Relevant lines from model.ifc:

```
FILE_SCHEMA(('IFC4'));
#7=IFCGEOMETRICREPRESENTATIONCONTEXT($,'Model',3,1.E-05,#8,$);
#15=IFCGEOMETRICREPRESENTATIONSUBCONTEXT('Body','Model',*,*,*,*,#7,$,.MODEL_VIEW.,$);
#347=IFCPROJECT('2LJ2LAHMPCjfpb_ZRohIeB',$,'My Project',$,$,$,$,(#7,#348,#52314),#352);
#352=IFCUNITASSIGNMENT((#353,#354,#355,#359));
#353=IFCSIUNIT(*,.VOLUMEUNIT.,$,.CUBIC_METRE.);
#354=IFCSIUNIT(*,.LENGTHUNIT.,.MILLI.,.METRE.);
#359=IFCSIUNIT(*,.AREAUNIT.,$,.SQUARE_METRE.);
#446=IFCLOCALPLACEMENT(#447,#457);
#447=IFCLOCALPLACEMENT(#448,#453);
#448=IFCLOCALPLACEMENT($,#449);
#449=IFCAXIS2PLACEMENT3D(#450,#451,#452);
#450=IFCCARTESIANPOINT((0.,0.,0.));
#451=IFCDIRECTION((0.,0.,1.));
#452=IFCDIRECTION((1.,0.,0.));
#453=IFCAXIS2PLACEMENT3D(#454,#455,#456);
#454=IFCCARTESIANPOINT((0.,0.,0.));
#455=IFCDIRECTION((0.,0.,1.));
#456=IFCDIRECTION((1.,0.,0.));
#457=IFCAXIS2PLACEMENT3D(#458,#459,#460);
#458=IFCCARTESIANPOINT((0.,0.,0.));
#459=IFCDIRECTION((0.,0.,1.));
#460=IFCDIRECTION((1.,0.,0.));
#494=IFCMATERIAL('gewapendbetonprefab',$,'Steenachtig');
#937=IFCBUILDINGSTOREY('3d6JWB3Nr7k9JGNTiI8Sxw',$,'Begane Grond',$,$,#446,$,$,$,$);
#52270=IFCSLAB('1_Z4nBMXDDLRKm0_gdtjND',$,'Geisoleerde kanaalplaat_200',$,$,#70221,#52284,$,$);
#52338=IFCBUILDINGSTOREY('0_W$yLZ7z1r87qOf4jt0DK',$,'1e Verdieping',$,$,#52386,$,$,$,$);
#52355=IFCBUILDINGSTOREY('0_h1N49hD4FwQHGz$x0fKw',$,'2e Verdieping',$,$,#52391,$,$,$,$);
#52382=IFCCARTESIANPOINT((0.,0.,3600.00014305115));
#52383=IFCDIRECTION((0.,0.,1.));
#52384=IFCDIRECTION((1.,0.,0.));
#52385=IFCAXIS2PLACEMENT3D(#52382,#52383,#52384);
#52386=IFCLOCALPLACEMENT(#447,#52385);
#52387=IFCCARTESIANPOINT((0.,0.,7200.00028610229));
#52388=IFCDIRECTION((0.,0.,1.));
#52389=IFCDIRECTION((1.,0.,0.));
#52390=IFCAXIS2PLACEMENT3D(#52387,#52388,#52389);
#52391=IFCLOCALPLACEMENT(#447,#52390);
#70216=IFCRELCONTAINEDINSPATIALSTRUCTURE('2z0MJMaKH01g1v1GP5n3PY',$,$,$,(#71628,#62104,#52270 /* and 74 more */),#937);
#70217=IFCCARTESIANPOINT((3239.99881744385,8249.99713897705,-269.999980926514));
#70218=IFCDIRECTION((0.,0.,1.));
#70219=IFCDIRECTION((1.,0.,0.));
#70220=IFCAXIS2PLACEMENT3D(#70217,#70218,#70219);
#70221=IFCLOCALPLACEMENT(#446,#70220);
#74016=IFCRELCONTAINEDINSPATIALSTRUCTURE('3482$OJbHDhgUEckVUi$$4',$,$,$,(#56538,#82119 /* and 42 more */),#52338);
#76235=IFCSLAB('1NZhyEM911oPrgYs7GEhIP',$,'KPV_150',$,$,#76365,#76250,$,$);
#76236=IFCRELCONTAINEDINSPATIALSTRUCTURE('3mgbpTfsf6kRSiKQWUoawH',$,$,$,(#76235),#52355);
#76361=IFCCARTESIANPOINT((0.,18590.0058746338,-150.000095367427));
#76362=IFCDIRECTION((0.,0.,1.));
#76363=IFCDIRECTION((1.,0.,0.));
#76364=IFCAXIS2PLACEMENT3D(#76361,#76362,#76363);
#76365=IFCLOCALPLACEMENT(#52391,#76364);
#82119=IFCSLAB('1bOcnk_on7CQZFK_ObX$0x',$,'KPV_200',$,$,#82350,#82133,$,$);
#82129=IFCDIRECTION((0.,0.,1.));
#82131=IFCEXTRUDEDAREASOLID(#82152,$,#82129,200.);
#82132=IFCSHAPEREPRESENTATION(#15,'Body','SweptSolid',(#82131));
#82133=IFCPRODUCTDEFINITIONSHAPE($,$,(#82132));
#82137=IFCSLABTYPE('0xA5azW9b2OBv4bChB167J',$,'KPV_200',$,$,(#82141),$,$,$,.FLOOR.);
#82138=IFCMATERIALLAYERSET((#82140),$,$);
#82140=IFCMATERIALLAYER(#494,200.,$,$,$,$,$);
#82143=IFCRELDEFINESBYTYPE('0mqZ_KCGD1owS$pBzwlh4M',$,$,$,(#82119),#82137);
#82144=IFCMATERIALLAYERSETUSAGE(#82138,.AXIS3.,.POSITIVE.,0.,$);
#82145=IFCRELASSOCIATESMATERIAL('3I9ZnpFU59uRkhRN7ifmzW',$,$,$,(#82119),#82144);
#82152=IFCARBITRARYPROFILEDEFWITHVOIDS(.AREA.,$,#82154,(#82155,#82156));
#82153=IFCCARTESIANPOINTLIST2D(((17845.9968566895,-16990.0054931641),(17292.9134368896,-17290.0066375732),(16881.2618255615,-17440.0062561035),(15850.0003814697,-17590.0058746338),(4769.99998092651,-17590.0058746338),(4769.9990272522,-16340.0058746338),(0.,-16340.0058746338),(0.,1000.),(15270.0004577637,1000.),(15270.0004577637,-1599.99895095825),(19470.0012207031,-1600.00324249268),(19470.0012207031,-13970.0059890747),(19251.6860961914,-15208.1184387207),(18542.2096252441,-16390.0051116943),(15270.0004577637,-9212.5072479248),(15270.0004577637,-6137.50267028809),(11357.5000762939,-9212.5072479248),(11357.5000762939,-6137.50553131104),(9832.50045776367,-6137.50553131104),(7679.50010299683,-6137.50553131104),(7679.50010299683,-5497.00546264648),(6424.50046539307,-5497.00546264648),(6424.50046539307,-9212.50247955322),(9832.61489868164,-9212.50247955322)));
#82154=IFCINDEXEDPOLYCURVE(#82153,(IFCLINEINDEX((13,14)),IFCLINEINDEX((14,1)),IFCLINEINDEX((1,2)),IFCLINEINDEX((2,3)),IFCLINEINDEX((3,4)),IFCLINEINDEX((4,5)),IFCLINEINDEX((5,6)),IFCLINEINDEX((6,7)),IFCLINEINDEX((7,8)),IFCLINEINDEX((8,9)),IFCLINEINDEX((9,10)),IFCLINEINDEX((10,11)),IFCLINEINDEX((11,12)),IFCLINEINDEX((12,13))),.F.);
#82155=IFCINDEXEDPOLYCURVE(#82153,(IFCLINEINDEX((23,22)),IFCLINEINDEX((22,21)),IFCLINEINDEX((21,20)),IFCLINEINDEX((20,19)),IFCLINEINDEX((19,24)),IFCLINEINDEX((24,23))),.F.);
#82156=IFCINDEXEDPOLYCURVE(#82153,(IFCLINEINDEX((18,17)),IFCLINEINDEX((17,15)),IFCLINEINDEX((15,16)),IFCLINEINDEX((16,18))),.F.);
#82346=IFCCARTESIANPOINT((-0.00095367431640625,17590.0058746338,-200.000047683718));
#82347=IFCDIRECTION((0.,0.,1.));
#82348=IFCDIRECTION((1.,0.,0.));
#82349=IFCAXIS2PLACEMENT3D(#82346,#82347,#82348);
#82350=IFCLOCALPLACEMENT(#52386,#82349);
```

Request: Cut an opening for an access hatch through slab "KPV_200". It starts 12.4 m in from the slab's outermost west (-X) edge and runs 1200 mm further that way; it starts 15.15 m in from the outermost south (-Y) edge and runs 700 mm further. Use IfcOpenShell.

```python
import numpy as np
import ifcopenshell
import ifcopenshell.api.feature
import ifcopenshell.api.geometry
import ifcopenshell.api.root
import ifcopenshell.geom
import ifcopenshell.util.placement
import ifcopenshell.util.representation
import ifcopenshell.util.shape
import ifcopenshell.util.unit

model = ifcopenshell.open("model.ifc")
unit_scale = ifcopenshell.util.unit.calculate_unit_scale(model)
settings = ifcopenshell.geom.settings()


def volume(element):
    """Net volume in cubic metres, openings subtracted."""
    shape = ifcopenshell.geom.create_shape(settings, element)
    return ifcopenshell.util.shape.get_volume(shape.geometry)


slab = model.by_guid("1bOcnk_on7CQZFK_ObX$0x")
before = volume(slab)

# Extent in the slab's own axes, in metres. The edges named are its -X and -Y sides.
slab_shape = ifcopenshell.geom.create_shape(settings, slab)
vertices = ifcopenshell.util.shape.get_vertices(slab_shape.geometry)
x_min, y_min, bottom = vertices.min(axis=0)
top = vertices[:, 2].max()

opening = ifcopenshell.api.root.create_entity(model, ifc_class="IfcOpeningElement", name="Access hatch opening", predefined_type="OPENING")
context = ifcopenshell.util.representation.get_context(model, "Model", "Body", "MODEL_VIEW")
width, depth = 1.2, 0.7
outline = [(0.0, 0.0), (width, 0.0), (width, depth), (0.0, depth), (0.0, 0.0)]
# Overshoot both faces by 50 mm so the cut is clean.
shape = ifcopenshell.api.geometry.add_slab_representation(
    model, context=context, depth=top - bottom + 0.1, polyline=outline
)
ifcopenshell.api.geometry.assign_representation(model, product=opening, representation=shape)

matrix = ifcopenshell.util.placement.get_local_placement(slab.ObjectPlacement)
matrix[:, 3] = matrix @ np.append(np.array([x_min + 12.4, y_min + 15.15, bottom - 0.05]) / unit_scale, 1.0)
ifcopenshell.api.geometry.edit_object_placement(model, product=opening, matrix=matrix, is_si=False)
ifcopenshell.api.feature.add_feature(model, feature=opening, element=slab)

after = volume(slab)

print(f"slab volume {before:.3f} -> {after:.3f} m3")

model.write("model_v2.ifc")
```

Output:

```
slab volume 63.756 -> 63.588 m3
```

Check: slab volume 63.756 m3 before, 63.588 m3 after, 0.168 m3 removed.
